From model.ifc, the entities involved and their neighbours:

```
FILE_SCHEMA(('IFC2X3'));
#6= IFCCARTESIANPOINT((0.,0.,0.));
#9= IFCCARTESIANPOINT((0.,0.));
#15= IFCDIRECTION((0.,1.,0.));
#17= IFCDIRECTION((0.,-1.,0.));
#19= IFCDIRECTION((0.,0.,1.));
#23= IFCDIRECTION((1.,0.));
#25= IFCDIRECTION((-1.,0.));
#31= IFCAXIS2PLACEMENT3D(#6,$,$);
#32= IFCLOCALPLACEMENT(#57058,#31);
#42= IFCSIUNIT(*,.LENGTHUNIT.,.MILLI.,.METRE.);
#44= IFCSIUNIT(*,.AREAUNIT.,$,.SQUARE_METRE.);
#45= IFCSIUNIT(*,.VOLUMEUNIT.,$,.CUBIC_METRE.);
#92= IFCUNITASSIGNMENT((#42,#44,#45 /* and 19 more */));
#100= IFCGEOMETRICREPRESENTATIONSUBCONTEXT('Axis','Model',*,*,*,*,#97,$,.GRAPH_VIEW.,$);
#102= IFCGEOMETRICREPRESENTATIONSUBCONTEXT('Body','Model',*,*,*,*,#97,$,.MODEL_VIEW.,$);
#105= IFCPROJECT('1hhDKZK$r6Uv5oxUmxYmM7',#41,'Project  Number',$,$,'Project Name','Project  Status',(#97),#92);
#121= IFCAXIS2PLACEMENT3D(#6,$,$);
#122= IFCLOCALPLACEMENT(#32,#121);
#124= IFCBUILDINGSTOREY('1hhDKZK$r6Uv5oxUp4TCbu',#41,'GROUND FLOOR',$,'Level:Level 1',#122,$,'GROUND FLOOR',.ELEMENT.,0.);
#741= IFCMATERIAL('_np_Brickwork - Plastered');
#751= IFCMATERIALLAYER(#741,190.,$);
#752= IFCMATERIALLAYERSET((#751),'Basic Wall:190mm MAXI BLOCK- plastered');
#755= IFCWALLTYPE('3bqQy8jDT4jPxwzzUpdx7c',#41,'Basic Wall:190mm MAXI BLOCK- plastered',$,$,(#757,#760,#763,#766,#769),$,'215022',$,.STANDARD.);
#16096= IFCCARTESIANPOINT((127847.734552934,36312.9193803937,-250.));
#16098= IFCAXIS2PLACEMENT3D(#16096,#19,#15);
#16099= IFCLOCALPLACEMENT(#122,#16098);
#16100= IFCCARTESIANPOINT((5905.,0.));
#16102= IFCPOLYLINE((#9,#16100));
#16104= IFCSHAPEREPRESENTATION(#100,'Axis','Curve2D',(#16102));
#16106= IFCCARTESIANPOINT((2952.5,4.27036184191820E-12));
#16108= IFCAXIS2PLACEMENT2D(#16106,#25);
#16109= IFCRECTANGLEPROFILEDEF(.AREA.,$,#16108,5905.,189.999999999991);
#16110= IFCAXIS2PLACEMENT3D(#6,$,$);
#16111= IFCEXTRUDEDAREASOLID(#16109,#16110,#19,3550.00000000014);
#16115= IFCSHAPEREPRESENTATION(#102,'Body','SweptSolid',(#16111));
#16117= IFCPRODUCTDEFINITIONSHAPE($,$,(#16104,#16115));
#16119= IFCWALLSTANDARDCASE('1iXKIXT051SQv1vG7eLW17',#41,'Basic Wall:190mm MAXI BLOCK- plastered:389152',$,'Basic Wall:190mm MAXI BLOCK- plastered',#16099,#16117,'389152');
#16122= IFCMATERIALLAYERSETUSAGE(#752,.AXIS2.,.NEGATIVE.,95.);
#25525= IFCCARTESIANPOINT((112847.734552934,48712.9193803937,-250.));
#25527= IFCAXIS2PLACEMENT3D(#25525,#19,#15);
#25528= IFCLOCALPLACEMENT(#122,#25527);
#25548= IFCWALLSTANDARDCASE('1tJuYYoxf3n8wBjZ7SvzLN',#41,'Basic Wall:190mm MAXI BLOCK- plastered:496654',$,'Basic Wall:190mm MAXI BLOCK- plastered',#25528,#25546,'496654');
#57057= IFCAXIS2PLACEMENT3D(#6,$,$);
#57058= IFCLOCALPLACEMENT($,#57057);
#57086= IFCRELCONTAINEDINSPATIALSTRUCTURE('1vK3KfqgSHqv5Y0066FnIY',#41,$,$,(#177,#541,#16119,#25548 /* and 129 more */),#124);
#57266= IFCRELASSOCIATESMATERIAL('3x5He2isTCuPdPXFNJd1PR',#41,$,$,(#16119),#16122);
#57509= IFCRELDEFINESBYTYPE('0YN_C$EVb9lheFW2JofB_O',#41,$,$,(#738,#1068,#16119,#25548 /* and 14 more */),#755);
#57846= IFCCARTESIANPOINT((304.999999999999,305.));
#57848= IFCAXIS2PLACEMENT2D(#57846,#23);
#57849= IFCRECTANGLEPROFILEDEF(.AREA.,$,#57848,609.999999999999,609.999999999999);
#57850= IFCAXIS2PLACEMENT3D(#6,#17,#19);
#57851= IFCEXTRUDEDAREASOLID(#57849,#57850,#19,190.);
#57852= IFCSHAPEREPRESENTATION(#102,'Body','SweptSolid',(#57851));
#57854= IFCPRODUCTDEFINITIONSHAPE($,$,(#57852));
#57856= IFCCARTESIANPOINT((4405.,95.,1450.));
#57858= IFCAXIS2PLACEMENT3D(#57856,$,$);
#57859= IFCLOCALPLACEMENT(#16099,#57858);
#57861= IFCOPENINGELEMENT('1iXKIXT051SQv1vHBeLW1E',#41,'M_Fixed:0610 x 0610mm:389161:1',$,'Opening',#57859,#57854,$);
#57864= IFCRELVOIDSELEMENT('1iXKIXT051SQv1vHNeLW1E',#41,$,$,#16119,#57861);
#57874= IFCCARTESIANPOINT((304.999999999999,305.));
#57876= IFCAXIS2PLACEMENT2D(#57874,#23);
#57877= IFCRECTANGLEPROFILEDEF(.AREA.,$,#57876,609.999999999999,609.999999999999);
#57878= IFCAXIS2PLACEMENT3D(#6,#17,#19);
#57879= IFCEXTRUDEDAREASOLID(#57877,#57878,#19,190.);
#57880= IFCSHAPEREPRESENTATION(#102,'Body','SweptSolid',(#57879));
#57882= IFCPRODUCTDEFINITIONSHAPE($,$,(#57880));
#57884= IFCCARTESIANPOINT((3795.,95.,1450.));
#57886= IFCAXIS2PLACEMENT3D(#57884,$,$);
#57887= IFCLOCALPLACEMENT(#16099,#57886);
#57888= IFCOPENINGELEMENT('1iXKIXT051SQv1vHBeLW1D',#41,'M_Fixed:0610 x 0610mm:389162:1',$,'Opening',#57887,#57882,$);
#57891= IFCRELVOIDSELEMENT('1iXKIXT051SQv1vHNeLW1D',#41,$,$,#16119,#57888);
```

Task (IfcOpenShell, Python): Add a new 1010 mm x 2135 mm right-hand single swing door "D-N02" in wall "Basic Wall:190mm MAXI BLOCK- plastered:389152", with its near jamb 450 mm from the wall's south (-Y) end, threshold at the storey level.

```python
import numpy as np
import ifcopenshell
import ifcopenshell.api.feature
import ifcopenshell.api.geometry
import ifcopenshell.api.root
import ifcopenshell.api.spatial
import ifcopenshell.api.type
import ifcopenshell.geom
import ifcopenshell.util.element
import ifcopenshell.util.placement
import ifcopenshell.util.representation
import ifcopenshell.util.shape
import ifcopenshell.util.unit

model = ifcopenshell.open("model.ifc")
unit_scale = ifcopenshell.util.unit.calculate_unit_scale(model)
settings = ifcopenshell.geom.settings()


def volume(element):
    """Net volume in cubic metres, openings subtracted."""
    shape = ifcopenshell.geom.create_shape(settings, element)
    return ifcopenshell.util.shape.get_volume(shape.geometry)


wall = model.by_guid("1iXKIXT051SQv1vG7eLW17")
storey = ifcopenshell.util.element.get_container(wall, ifc_class="IfcBuildingStorey")
context = ifcopenshell.util.representation.get_context(model, "Model", "Body", "MODEL_VIEW")
before = volume(wall)

width, height, from_end, sill = 1.01, 2.135, 0.45, 0.0  # metres

# The wall runs along its own X axis, and the end named is its -X end.
wall_shape = ifcopenshell.geom.create_shape(settings, wall)
x, y, z = ifcopenshell.util.shape.get_vertices(wall_shape.geometry).T
start = x.min() + from_end
face, thickness = float(y.min()), float(y.max() - y.min())
wall_matrix = ifcopenshell.util.placement.get_local_placement(wall.ObjectPlacement)
level = ifcopenshell.util.placement.get_local_placement(storey.ObjectPlacement)[2, 3]


def in_wall(x, y):
    """Placement at x, y metres in the wall's axes, at sill height."""
    matrix = wall_matrix.copy()
    matrix[:, 3] = wall_matrix @ np.array([x / unit_scale, y / unit_scale, 0.0, 1.0])
    matrix[2, 3] = level + sill / unit_scale
    return matrix


# Opening: a box that overshoots both wall faces by 50 mm.
opening = ifcopenshell.api.root.create_entity(model, ifc_class="IfcOpeningElement")
box = ifcopenshell.api.geometry.add_wall_representation(
    model, context=context, length=width, height=height, thickness=thickness + 0.1
)
ifcopenshell.api.geometry.assign_representation(model, product=opening, representation=box)
ifcopenshell.api.geometry.edit_object_placement(model, product=opening, matrix=in_wall(start, face - 0.05), is_si=False)
ifcopenshell.api.feature.add_feature(model, feature=opening, element=wall)

door = ifcopenshell.api.root.create_entity(model, ifc_class="IfcDoor", name="D-N02")
door.OverallWidth, door.OverallHeight = width / unit_scale, height / unit_scale
body = ifcopenshell.api.geometry.add_door_representation(
    model,
    context=context,
    overall_width=door.OverallWidth,
    overall_height=door.OverallHeight,
    operation_type="SINGLE_SWING_RIGHT",
    lining_properties={"LiningDepth": thickness / unit_scale, "ThresholdDepth": thickness / unit_scale},
)
ifcopenshell.api.geometry.assign_representation(model, product=door, representation=body)
ifcopenshell.api.spatial.assign_container(model, products=[door], relating_structure=storey)
fills = ifcopenshell.api.feature.add_filling(model, opening=opening, element=door)
fills.OwnerHistory = door.OwnerHistory  # required in IFC2X3

# IFC2X3 keeps the operation on the door style.
style = ifcopenshell.api.root.create_entity(model, ifc_class="IfcDoorStyle", name="D-N02")
style.OperationType, style.ConstructionType = "SINGLE_SWING_RIGHT", "NOTDEFINED"
style.ParameterTakesPrecedence = style.Sizeable = False
ifcopenshell.api.type.assign_type(model, related_objects=[door], relating_type=style)

# The lining spans the wall, so the door starts at the wall face.
ifcopenshell.api.geometry.edit_object_placement(model, product=door, matrix=in_wall(start, face), is_si=False)

after = volume(wall)

print(f"wall volume {before:.3f} -> {after:.3f} m3")

model.write("model-out.ifc")
```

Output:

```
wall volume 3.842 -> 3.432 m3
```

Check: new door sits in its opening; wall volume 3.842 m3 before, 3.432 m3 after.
